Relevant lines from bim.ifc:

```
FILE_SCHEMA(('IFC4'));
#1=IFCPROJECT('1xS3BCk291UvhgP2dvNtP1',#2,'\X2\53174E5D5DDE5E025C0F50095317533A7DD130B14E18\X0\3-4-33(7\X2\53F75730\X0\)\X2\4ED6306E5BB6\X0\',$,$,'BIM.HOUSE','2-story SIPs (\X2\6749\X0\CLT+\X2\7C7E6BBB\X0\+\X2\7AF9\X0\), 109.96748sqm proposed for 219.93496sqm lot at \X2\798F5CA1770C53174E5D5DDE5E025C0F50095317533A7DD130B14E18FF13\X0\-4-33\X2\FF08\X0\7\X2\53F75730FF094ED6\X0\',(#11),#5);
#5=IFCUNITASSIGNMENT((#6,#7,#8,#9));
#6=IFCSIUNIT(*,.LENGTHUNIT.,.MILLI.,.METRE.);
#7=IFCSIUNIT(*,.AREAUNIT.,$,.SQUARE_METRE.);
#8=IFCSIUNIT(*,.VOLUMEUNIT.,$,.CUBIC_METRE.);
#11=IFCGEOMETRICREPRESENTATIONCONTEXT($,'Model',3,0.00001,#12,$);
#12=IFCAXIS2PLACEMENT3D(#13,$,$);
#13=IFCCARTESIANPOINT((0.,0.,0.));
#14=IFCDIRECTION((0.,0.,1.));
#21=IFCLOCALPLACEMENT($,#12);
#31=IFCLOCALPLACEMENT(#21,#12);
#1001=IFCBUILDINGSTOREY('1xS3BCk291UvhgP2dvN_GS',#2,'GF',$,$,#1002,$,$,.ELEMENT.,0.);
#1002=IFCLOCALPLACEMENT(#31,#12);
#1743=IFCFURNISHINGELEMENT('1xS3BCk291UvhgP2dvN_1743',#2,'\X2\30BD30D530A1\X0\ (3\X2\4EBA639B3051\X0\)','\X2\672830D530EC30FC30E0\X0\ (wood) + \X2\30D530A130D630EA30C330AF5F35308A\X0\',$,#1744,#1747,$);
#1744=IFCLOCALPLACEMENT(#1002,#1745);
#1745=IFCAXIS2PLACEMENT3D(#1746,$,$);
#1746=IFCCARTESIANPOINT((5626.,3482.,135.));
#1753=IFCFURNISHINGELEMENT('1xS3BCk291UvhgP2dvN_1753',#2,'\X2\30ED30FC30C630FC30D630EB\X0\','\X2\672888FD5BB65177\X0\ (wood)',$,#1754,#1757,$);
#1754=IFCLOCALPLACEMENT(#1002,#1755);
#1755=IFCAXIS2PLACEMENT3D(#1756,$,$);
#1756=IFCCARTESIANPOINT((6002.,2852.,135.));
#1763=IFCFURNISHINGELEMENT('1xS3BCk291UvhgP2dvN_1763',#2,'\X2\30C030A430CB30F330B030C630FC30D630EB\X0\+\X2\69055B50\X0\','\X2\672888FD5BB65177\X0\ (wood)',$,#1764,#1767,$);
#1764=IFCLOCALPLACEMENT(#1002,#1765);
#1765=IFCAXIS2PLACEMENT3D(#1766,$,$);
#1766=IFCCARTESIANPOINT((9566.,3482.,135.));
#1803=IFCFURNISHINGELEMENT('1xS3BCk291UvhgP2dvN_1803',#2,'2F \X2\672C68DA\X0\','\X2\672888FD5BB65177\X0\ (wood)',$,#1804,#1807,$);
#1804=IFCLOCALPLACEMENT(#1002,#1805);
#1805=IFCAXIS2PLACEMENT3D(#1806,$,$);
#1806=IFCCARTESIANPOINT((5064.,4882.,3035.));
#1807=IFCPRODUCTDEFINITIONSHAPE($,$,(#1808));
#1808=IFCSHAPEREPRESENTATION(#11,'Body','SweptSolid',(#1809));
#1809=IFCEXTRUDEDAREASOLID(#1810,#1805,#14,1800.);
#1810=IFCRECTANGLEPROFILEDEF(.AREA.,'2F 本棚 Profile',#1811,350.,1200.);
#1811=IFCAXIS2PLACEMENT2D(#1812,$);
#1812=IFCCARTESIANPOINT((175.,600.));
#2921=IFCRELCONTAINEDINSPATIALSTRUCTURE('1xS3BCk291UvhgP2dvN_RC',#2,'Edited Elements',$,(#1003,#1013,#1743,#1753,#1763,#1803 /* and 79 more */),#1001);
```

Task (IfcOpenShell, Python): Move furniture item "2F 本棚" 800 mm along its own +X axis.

```python
import ifcopenshell
import ifcopenshell.api.geometry
import ifcopenshell.util.placement
import ifcopenshell.util.unit

model = ifcopenshell.open("bim.ifc")
unit_scale = ifcopenshell.util.unit.calculate_unit_scale(model)

item = model.by_guid("1xS3BCk291UvhgP2dvN_1803")
matrix = ifcopenshell.util.placement.get_local_placement(item.ObjectPlacement)
matrix[:3, 3] += matrix[:3, 0] * 0.8 / unit_scale
ifcopenshell.api.geometry.edit_object_placement(model, product=item, matrix=matrix, is_si=False)

print(ifcopenshell.util.placement.get_local_placement(item.ObjectPlacement).round(3) + 0.0)

model.write("bim_v2.ifc")
```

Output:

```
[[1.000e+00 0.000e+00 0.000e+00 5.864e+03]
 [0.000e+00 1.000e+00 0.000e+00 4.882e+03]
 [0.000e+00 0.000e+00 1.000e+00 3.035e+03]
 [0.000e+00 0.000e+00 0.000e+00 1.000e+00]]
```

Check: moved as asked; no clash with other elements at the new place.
